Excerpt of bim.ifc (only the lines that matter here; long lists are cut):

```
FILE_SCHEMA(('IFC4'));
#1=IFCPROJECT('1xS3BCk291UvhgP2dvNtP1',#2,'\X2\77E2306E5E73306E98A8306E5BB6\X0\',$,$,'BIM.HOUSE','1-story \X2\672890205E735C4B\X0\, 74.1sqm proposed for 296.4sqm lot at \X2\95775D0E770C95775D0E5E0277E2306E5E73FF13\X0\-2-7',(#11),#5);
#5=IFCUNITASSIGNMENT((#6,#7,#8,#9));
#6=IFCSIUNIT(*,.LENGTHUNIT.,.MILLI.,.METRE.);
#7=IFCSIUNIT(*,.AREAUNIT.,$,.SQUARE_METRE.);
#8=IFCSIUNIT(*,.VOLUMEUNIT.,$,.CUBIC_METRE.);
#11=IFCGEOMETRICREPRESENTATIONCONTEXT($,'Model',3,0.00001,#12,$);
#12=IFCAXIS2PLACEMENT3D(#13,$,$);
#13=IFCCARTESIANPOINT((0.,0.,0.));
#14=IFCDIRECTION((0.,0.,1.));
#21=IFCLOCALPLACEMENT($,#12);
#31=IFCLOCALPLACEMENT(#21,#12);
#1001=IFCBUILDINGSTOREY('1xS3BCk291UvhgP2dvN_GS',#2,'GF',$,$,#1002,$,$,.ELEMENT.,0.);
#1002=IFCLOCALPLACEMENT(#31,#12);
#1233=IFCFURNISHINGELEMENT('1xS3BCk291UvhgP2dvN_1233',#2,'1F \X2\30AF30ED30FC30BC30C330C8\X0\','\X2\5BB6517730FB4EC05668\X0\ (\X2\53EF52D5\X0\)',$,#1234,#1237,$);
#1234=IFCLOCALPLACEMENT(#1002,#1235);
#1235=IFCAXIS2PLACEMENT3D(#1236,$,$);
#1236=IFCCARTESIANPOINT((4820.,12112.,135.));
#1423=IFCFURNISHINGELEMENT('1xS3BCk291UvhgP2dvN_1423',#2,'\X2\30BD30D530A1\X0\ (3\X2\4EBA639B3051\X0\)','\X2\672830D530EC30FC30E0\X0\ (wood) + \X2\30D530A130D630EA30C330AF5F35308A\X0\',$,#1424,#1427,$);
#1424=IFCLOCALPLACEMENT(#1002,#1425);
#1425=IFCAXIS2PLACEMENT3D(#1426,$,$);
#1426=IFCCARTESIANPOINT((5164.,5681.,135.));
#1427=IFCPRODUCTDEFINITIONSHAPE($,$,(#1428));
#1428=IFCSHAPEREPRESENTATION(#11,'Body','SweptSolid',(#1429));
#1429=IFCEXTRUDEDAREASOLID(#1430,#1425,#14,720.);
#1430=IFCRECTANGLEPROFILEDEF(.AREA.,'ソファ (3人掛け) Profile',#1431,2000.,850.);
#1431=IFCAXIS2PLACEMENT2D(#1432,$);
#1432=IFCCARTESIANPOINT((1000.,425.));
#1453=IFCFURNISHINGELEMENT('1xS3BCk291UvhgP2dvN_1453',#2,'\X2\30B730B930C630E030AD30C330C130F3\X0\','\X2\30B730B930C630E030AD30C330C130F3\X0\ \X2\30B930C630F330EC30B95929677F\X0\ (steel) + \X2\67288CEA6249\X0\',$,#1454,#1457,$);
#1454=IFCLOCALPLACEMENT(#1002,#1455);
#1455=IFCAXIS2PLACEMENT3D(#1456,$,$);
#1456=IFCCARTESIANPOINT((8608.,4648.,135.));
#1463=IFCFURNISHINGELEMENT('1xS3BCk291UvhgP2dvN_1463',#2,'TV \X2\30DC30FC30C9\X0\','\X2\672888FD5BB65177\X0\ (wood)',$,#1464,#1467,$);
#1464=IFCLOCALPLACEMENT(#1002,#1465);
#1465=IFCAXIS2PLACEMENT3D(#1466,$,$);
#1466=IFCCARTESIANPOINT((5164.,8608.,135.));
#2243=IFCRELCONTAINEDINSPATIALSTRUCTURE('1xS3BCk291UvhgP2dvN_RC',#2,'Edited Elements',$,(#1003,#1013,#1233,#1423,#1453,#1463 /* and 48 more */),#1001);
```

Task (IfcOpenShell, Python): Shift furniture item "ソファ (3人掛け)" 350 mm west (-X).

```python
import ifcopenshell
import ifcopenshell.api.geometry
import ifcopenshell.util.placement

model = ifcopenshell.open("bim.ifc")

item = model.by_guid("1xS3BCk291UvhgP2dvN_1423")
matrix = ifcopenshell.util.placement.get_local_placement(item.ObjectPlacement)
matrix[0, 3] -= 350.0
ifcopenshell.api.geometry.edit_object_placement(model, product=item, matrix=matrix, is_si=False)

print(ifcopenshell.util.placement.get_local_placement(item.ObjectPlacement).round(3) + 0.0)

model.write("bim_edited.ifc")
```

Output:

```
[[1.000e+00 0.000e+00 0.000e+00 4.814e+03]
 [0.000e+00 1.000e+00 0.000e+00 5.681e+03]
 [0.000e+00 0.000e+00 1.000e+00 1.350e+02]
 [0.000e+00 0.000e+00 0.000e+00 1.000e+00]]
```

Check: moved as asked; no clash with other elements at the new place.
